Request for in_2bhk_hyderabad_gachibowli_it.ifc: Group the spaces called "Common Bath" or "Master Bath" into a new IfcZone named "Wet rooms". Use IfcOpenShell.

First a look at what the model holds.

```python
import ifcopenshell

model = ifcopenshell.open("in_2bhk_hyderabad_gachibowli_it.ifc")
print(model.schema)
seen = {}
for space in model.by_type("IfcSpace"):
    seen[space.LongName] = seen.get(space.LongName, 0) + 1
for name, count in sorted(seen.items(), key=str):
    print(count, "x", name)
print("zones:", [z.Name for z in model.by_type("IfcZone")][:20])
```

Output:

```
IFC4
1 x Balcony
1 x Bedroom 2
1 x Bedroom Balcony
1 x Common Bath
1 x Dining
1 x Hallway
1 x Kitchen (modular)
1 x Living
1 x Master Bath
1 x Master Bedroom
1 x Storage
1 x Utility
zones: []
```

```python
import ifcopenshell
import ifcopenshell.api.group
import ifcopenshell.api.root

model = ifcopenshell.open("in_2bhk_hyderabad_gachibowli_it.ifc")

names = {"Common Bath", "Master Bath"}
spaces = [s for s in model.by_type("IfcSpace") if s.LongName in names]

zone = ifcopenshell.api.root.create_entity(model, ifc_class="IfcZone", name="Wet rooms")
ifcopenshell.api.group.assign_group(model, products=spaces, group=zone)
print(len(spaces), "spaces in", zone.Name)

model.write("in_2bhk_hyderabad_gachibowli_it_updated.ifc")
```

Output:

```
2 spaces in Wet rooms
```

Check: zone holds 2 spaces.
